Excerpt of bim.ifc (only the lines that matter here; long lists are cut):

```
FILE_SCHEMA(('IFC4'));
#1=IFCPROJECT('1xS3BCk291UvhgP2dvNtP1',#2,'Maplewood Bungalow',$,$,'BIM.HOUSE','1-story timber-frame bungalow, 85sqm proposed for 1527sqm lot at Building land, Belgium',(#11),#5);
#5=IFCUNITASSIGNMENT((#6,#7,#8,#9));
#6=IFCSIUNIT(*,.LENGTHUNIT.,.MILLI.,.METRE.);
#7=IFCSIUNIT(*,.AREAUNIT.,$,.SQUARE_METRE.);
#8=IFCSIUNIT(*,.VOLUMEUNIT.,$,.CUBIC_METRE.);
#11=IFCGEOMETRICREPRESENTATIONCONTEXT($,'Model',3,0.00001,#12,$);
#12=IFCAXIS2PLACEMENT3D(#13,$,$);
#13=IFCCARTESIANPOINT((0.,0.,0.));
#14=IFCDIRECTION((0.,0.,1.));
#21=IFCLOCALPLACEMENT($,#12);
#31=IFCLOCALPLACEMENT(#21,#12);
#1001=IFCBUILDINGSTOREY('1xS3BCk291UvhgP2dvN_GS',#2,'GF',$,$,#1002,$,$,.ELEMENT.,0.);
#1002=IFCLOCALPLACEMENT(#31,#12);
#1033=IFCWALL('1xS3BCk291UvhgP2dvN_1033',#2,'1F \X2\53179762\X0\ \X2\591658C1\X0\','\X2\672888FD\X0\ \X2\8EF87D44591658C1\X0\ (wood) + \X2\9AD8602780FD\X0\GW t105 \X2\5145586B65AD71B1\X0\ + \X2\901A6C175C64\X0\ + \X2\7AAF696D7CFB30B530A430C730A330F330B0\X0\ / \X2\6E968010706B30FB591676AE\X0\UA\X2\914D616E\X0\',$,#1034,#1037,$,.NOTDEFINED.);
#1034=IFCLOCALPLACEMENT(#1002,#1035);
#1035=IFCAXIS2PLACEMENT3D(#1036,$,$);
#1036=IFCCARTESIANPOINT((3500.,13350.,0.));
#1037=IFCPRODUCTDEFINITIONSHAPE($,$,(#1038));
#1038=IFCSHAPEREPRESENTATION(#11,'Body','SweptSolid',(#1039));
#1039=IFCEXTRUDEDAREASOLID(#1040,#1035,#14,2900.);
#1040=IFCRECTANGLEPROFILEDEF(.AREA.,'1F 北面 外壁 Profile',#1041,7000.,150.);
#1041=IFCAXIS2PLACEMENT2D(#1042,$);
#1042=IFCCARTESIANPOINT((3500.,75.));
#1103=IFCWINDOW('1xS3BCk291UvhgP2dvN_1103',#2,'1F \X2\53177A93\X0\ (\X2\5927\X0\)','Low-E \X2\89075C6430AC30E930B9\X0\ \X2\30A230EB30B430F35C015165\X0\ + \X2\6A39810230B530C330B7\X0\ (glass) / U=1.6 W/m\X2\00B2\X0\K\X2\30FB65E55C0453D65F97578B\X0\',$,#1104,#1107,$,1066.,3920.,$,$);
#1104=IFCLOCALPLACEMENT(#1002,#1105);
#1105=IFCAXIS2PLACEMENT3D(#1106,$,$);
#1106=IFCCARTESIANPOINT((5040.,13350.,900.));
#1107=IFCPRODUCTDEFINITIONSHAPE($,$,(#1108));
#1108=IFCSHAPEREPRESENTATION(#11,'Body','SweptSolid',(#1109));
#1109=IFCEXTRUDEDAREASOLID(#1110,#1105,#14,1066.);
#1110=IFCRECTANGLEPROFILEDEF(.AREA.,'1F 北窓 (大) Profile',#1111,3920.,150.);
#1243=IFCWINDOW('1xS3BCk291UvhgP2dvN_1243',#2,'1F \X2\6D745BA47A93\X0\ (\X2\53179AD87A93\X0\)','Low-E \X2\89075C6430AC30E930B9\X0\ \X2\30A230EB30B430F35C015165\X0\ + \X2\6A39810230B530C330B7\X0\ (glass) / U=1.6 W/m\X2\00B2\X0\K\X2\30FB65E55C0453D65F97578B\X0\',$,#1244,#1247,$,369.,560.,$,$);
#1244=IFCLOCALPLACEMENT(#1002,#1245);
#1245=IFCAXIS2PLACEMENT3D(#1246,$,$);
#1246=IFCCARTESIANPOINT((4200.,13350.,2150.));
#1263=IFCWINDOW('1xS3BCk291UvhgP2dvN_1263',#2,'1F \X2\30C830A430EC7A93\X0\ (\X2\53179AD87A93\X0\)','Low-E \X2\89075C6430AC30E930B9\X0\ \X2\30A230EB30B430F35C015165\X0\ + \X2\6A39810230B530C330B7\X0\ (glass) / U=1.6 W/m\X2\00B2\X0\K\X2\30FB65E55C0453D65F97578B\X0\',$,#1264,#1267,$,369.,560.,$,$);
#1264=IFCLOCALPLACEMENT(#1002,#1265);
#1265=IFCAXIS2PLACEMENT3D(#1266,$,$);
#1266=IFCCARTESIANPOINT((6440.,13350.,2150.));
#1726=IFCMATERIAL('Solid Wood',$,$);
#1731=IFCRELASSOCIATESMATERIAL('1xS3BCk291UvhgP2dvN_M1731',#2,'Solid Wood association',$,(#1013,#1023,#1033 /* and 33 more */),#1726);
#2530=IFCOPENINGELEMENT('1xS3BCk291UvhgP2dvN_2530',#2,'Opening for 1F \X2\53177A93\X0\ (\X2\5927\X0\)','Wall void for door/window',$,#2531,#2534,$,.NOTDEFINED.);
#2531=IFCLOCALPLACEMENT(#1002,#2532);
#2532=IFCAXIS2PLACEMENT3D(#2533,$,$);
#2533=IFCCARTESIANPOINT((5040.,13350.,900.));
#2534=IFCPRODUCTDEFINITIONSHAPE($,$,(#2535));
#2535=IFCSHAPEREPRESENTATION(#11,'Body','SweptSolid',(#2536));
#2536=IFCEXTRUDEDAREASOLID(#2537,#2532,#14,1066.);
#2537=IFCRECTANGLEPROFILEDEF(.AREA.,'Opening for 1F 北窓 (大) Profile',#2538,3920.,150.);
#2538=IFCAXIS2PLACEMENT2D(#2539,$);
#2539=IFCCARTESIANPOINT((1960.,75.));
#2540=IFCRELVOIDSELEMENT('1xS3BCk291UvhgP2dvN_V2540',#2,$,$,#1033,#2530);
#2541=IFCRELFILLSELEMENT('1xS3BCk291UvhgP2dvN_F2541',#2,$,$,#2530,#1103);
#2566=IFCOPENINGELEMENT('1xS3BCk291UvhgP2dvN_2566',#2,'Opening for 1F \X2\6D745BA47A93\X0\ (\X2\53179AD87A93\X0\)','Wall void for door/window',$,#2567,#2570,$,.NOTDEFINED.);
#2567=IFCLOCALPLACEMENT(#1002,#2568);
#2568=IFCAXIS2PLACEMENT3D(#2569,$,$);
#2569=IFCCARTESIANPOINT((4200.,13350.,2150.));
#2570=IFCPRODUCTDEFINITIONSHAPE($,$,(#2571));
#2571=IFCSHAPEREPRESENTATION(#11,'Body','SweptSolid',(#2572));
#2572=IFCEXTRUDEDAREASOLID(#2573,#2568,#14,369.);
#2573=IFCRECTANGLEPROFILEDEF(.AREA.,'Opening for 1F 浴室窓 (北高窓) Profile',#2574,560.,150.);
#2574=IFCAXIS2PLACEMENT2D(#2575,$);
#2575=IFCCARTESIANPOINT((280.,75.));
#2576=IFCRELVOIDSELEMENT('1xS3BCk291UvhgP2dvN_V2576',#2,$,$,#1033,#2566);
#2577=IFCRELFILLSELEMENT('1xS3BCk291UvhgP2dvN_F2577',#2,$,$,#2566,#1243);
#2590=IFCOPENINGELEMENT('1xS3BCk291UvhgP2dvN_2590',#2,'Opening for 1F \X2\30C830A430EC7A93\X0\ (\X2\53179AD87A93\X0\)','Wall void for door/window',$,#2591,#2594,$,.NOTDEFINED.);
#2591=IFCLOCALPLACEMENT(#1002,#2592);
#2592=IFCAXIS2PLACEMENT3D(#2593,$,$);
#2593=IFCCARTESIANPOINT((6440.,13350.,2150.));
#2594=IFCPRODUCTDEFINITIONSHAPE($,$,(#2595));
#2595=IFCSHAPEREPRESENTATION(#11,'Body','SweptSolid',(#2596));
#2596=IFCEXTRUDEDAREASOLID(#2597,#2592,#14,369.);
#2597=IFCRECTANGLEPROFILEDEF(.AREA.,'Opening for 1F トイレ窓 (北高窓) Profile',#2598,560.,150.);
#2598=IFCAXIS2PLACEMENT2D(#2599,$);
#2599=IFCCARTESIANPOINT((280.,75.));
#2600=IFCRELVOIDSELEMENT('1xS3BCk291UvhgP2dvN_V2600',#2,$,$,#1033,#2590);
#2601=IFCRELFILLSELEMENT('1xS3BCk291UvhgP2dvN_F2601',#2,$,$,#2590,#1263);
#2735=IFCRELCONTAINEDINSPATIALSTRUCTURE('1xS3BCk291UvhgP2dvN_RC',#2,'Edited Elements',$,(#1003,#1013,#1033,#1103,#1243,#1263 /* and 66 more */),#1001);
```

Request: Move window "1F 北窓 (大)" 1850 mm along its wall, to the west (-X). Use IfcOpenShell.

```python
import ifcopenshell
import ifcopenshell.api.geometry
import ifcopenshell.util.placement
import ifcopenshell.util.unit

model = ifcopenshell.open("bim.ifc")
unit_scale = ifcopenshell.util.unit.calculate_unit_scale(model)

window = model.by_id(1103)
opening = window.FillsVoids[0].RelatingOpeningElement
wall = opening.VoidsElements[0].RelatingBuildingElement

wall_matrix = ifcopenshell.util.placement.get_local_placement(wall.ObjectPlacement)
shift = wall_matrix[:3, 0] * -1.85 / unit_scale
before = ifcopenshell.util.placement.get_local_placement(window.ObjectPlacement)[:3, 3].copy()

# The window is not placed relative to its opening, so move both.
for product in (opening, window):
    matrix = ifcopenshell.util.placement.get_local_placement(product.ObjectPlacement)
    matrix[:3, 3] += shift
    ifcopenshell.api.geometry.edit_object_placement(model, product=product, matrix=matrix, is_si=False)

after = ifcopenshell.util.placement.get_local_placement(window.ObjectPlacement)[:3, 3]
print("window moved by", (after - before).round(3) + 0.0)

model.write("bim_updated.ifc")
```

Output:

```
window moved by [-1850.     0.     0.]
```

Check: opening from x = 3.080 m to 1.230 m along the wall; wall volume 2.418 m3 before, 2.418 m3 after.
